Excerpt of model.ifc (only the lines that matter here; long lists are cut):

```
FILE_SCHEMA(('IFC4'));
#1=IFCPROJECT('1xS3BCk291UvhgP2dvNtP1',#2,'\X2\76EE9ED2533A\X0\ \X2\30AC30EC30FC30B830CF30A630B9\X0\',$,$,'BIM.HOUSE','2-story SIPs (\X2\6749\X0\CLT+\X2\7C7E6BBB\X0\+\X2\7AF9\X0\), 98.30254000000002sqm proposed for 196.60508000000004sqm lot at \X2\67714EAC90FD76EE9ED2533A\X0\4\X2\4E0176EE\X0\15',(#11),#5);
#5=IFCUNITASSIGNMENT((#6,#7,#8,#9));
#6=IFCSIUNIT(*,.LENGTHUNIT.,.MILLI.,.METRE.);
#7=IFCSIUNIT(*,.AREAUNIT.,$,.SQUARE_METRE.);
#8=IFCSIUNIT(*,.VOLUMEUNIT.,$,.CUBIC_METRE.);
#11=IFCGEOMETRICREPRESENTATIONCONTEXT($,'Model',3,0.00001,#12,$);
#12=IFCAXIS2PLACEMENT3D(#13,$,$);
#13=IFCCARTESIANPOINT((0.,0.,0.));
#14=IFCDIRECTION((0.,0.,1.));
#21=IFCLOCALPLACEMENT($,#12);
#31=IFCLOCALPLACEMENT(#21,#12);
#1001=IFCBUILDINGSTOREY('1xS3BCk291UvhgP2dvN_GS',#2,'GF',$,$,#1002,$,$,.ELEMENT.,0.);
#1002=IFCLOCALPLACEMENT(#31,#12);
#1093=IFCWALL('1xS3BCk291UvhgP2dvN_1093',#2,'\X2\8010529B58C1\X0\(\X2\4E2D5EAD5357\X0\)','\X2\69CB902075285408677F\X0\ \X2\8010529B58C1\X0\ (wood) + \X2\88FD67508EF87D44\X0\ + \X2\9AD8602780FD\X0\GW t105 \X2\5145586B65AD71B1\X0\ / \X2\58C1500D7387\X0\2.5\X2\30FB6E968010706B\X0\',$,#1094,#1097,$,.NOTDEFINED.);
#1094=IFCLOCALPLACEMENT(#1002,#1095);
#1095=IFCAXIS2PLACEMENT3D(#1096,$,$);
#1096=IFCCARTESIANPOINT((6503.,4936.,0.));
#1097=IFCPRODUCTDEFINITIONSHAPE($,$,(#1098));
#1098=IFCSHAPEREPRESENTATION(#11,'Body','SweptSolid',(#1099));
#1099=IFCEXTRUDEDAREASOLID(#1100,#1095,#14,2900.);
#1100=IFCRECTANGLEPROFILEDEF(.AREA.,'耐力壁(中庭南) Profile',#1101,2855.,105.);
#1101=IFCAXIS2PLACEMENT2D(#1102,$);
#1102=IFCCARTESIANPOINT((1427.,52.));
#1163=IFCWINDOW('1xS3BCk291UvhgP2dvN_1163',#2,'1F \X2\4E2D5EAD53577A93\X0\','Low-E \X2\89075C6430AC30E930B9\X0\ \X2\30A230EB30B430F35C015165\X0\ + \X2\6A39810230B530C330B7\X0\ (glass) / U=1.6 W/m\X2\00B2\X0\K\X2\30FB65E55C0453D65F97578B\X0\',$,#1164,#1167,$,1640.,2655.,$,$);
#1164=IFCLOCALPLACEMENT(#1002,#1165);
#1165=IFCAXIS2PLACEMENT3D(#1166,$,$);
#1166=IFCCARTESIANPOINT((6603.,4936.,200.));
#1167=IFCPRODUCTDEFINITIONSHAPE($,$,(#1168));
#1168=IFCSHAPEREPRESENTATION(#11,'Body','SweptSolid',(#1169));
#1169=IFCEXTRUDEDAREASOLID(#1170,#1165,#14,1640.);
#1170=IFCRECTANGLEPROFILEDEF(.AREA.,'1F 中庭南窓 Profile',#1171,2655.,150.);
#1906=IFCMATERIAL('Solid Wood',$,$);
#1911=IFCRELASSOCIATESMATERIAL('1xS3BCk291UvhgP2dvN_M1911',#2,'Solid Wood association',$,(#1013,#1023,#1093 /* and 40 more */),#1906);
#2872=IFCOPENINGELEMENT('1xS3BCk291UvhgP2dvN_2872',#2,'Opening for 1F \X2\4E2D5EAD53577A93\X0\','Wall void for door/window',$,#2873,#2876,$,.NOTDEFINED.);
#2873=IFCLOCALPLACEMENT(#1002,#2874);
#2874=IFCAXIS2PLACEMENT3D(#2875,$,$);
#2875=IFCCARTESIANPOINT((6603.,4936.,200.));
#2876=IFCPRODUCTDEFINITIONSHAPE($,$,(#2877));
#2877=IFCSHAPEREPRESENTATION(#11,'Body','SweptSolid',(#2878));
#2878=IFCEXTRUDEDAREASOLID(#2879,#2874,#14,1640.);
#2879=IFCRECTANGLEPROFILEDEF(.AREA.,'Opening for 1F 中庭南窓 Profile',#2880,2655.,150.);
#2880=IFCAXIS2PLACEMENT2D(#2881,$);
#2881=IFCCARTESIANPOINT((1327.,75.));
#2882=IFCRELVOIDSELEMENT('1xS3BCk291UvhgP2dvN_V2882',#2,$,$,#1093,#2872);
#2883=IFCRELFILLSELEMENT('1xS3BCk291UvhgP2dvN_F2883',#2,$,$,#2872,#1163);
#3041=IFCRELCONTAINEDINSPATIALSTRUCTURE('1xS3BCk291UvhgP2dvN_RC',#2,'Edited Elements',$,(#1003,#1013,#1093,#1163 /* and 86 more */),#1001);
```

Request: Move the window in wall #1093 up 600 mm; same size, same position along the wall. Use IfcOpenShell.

```python
import numpy as np
import ifcopenshell
import ifcopenshell.api.geometry
import ifcopenshell.util.placement
import ifcopenshell.util.unit

model = ifcopenshell.open("model.ifc")
unit_scale = ifcopenshell.util.unit.calculate_unit_scale(model)

window = model.by_guid("1xS3BCk291UvhgP2dvN_1163")
opening = window.FillsVoids[0].RelatingOpeningElement
dz = 0.6 / unit_scale

shift = np.array([0.0, 0.0, dz])
# The window is not placed relative to its opening, so move both.
for product in (opening, window):
    matrix = ifcopenshell.util.placement.get_local_placement(product.ObjectPlacement)
    matrix[:3, 3] += shift
    ifcopenshell.api.geometry.edit_object_placement(model, product=product, matrix=matrix, is_si=False)

print(f"moved by {dz * unit_scale:+.3f} m")

model.write("model_updated.ifc")
```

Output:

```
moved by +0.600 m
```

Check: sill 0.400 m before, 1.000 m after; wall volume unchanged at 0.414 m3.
